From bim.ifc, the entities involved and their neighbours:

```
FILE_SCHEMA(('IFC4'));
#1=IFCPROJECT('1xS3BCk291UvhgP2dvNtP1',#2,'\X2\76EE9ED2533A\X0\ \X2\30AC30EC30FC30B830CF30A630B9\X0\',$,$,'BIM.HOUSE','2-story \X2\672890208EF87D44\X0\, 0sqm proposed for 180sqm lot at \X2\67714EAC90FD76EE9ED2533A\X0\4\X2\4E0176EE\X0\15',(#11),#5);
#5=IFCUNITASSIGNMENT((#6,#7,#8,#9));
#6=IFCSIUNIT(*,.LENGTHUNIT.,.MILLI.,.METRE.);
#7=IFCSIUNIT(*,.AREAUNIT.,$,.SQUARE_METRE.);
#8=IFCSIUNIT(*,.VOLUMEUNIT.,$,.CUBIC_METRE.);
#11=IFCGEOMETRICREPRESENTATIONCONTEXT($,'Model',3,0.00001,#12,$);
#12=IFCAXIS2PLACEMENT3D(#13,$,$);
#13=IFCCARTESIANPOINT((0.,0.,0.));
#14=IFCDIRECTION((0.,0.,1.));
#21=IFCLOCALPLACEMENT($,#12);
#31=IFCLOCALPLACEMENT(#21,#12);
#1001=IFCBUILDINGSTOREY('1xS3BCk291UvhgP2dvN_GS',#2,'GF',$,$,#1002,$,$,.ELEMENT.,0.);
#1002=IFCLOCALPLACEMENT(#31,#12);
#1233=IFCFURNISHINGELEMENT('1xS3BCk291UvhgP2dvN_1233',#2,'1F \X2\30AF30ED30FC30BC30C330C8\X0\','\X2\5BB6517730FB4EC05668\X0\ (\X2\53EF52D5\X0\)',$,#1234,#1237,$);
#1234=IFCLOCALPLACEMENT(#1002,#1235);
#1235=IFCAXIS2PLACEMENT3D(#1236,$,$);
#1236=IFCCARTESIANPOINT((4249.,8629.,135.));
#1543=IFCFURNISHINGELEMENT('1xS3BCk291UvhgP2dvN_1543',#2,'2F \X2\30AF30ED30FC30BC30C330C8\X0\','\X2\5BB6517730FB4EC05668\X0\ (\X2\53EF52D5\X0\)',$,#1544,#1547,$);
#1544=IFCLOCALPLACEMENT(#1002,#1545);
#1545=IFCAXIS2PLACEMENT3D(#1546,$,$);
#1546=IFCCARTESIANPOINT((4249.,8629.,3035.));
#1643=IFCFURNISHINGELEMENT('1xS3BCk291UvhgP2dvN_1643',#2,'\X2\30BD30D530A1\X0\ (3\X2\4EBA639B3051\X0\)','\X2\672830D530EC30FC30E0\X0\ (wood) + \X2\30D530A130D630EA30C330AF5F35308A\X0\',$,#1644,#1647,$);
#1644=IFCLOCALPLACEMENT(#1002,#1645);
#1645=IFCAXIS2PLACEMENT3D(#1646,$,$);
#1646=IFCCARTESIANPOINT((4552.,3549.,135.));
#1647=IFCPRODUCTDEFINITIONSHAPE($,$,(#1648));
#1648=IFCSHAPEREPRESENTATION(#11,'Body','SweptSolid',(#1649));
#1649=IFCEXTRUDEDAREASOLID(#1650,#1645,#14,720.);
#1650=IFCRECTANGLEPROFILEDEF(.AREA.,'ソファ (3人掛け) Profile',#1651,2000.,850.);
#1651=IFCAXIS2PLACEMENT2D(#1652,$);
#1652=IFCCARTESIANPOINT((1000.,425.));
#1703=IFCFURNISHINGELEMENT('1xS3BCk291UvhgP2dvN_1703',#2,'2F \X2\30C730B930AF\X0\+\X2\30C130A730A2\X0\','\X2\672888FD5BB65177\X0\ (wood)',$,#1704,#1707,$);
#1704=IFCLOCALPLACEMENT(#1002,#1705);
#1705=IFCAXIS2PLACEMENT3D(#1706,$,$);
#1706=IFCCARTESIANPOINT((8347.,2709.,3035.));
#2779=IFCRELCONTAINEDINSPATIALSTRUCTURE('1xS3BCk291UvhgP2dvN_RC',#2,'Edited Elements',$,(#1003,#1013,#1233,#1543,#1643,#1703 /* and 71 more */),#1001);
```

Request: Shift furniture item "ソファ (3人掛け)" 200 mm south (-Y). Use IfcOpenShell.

```python
import ifcopenshell
import ifcopenshell.api.geometry
import ifcopenshell.util.placement

model = ifcopenshell.open("bim.ifc")

item = model.by_guid("1xS3BCk291UvhgP2dvN_1643")
matrix = ifcopenshell.util.placement.get_local_placement(item.ObjectPlacement)
matrix[1, 3] -= 200.0
ifcopenshell.api.geometry.edit_object_placement(model, product=item, matrix=matrix, is_si=False)

print(ifcopenshell.util.placement.get_local_placement(item.ObjectPlacement).round(3) + 0.0)

model.write("bim_edited.ifc")
```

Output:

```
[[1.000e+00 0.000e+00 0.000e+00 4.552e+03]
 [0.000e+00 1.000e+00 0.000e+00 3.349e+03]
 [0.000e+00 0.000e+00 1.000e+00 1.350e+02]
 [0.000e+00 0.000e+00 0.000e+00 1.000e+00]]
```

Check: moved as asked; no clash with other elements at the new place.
